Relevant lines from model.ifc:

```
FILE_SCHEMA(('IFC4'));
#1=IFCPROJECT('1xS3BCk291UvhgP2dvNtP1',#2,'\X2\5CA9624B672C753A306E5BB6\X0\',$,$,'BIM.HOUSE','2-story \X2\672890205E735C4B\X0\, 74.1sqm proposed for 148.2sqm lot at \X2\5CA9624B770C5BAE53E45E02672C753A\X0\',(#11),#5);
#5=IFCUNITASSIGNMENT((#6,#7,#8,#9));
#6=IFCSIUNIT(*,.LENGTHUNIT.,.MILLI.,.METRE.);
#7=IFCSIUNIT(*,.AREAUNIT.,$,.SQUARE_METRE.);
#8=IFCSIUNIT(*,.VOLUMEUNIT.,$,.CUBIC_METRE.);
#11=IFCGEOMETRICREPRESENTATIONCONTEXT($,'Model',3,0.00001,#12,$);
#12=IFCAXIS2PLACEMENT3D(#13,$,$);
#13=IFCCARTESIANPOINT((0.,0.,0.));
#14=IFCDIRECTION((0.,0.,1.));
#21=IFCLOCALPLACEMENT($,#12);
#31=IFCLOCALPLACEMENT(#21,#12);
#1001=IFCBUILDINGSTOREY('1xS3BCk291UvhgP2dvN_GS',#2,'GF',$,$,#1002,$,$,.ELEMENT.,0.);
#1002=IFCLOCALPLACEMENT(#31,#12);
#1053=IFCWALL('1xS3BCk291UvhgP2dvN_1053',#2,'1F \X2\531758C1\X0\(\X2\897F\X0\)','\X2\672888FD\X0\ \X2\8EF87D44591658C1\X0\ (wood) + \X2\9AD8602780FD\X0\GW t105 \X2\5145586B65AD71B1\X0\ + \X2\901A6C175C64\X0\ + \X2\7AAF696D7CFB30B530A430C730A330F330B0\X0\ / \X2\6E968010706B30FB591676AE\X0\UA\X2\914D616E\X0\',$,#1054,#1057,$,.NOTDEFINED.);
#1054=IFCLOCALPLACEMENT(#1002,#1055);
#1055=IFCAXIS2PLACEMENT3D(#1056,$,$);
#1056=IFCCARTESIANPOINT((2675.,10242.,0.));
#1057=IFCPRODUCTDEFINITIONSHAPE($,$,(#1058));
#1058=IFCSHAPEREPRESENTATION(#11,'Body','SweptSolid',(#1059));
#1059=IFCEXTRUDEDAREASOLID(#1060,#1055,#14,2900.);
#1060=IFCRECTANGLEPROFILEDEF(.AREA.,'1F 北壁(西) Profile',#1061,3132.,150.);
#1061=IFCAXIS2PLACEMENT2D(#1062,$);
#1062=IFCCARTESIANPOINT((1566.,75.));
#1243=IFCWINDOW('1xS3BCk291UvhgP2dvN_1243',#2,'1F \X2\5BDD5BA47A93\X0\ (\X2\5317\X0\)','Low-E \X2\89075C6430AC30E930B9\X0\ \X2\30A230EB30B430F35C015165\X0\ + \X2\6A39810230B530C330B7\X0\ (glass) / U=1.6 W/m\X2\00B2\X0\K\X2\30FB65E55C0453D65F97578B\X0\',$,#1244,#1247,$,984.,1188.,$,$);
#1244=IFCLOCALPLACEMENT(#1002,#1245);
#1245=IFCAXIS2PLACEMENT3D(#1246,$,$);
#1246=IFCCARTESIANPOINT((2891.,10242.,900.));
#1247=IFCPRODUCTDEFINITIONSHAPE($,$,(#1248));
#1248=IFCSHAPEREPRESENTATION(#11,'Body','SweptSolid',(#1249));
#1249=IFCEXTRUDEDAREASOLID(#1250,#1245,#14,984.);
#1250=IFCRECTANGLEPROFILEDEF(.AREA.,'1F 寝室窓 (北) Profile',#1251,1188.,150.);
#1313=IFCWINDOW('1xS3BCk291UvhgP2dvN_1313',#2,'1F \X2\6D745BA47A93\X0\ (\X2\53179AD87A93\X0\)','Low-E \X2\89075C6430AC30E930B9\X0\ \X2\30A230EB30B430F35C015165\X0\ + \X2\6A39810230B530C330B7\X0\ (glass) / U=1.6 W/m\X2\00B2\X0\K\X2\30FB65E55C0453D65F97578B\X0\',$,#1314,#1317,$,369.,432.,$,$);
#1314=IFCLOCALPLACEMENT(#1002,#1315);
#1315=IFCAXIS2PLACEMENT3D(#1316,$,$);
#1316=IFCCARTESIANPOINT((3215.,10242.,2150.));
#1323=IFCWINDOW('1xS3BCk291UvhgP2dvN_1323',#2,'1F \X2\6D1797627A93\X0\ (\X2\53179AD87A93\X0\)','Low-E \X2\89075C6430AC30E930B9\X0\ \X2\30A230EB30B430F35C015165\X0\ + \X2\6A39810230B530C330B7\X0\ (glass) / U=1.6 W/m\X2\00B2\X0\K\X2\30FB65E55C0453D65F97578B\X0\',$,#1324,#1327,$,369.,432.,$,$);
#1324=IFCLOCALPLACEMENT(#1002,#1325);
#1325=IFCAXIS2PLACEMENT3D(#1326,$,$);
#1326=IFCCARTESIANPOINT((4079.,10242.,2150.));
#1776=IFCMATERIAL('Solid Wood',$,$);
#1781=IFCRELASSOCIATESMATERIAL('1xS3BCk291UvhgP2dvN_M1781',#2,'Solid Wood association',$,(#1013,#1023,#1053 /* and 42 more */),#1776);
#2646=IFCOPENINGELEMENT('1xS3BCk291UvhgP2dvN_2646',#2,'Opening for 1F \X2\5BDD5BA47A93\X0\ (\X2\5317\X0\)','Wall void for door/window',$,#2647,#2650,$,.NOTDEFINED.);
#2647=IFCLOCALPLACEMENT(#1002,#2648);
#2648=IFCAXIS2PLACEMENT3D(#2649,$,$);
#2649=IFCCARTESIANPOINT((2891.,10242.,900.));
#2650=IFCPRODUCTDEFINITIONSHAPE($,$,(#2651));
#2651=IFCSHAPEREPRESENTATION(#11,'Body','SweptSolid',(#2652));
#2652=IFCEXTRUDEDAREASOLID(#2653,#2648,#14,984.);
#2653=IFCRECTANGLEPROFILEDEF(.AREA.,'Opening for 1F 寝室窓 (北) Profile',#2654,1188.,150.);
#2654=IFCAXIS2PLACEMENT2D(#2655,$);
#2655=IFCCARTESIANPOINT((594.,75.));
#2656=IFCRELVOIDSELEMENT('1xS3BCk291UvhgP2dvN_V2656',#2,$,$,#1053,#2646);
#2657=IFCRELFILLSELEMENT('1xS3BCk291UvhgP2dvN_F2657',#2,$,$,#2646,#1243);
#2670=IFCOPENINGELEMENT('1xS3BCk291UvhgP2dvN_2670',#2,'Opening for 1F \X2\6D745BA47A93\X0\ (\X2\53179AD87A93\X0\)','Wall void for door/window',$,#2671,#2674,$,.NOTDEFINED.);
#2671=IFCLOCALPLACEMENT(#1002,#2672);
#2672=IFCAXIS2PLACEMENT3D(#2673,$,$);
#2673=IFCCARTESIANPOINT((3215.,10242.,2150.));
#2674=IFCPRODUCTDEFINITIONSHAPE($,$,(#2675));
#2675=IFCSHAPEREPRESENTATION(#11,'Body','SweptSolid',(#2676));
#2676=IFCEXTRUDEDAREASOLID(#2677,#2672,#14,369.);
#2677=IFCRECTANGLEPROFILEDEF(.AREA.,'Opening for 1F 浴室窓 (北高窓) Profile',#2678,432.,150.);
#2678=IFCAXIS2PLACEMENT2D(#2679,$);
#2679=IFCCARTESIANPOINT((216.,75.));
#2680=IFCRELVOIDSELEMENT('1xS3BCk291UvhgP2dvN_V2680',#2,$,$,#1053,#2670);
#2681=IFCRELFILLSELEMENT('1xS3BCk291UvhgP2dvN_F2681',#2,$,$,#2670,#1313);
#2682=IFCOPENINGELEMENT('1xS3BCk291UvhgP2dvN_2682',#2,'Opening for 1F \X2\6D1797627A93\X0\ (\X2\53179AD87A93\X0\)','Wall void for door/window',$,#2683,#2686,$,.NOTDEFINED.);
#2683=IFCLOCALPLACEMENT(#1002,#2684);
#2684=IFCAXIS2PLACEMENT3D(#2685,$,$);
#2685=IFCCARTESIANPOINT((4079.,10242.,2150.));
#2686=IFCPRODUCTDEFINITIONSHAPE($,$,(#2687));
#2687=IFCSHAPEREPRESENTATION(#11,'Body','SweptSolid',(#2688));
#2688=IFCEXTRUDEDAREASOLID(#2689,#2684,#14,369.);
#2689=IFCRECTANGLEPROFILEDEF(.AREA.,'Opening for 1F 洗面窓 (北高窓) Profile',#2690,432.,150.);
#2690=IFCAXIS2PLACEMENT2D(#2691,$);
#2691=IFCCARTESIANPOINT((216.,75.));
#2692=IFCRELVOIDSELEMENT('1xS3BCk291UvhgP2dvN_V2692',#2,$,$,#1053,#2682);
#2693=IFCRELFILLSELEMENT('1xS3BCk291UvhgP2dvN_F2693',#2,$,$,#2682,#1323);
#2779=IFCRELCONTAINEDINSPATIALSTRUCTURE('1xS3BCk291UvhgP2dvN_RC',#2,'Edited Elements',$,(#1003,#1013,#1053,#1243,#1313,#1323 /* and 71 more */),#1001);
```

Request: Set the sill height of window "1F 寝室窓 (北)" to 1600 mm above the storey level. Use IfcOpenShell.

```python
import numpy as np
import ifcopenshell
import ifcopenshell.api.geometry
import ifcopenshell.geom
import ifcopenshell.util.element
import ifcopenshell.util.placement
import ifcopenshell.util.shape
import ifcopenshell.util.unit

model = ifcopenshell.open("model.ifc")
unit_scale = ifcopenshell.util.unit.calculate_unit_scale(model)

window = model.by_id(1243)
opening = window.FillsVoids[0].RelatingOpeningElement
storey = ifcopenshell.util.element.get_container(window, ifc_class="IfcBuildingStorey")
level = ifcopenshell.util.placement.get_local_placement(storey.ObjectPlacement)[2, 3]

# The opening's origin need not be at the sill, so measure its lowest point.
shape = ifcopenshell.geom.create_shape(ifcopenshell.geom.settings(), opening)
bottom = ifcopenshell.util.shape.get_shape_bottom_elevation(shape, shape.geometry) / unit_scale
dz = level + 1.6 / unit_scale - bottom

shift = np.array([0.0, 0.0, dz])
# The window is not placed relative to its opening, so move both.
for product in (opening, window):
    matrix = ifcopenshell.util.placement.get_local_placement(product.ObjectPlacement)
    matrix[:3, 3] += shift
    ifcopenshell.api.geometry.edit_object_placement(model, product=product, matrix=matrix, is_si=False)

print(f"moved by {dz * unit_scale:+.3f} m")

model.write("model_updated.ifc")
```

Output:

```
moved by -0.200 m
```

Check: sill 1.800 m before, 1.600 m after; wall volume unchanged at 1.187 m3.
